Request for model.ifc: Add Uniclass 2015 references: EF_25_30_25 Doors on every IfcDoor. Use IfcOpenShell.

First a look at what the model holds.

```python
import ifcopenshell

model = ifcopenshell.open("model.ifc")
print(model.schema)
print("classifications:", [c.Name for c in model.by_type("IfcClassification")])
for ifc_class in ("IfcDoor", "IfcRoof", "IfcStair", "IfcWall", "IfcWindow"):
    print(ifc_class, len(model.by_type(ifc_class)))
```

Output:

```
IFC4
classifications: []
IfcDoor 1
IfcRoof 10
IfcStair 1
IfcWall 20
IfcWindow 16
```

```python
import ifcopenshell
import ifcopenshell.api.classification

model = ifcopenshell.open("model.ifc")

system = ifcopenshell.api.classification.add_classification(model, classification="Uniclass 2015")

codes = {
    "IfcDoor": ("EF_25_30_25", "Doors"),
}
for ifc_class, (code, name) in codes.items():
    products = model.by_type(ifc_class)
    ifcopenshell.api.classification.add_reference(
        model, products=products, classification=system, identification=code, name=name
    )
    print(code, len(products))

model.write("model-out.ifc")
```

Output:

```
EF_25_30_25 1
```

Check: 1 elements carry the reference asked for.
